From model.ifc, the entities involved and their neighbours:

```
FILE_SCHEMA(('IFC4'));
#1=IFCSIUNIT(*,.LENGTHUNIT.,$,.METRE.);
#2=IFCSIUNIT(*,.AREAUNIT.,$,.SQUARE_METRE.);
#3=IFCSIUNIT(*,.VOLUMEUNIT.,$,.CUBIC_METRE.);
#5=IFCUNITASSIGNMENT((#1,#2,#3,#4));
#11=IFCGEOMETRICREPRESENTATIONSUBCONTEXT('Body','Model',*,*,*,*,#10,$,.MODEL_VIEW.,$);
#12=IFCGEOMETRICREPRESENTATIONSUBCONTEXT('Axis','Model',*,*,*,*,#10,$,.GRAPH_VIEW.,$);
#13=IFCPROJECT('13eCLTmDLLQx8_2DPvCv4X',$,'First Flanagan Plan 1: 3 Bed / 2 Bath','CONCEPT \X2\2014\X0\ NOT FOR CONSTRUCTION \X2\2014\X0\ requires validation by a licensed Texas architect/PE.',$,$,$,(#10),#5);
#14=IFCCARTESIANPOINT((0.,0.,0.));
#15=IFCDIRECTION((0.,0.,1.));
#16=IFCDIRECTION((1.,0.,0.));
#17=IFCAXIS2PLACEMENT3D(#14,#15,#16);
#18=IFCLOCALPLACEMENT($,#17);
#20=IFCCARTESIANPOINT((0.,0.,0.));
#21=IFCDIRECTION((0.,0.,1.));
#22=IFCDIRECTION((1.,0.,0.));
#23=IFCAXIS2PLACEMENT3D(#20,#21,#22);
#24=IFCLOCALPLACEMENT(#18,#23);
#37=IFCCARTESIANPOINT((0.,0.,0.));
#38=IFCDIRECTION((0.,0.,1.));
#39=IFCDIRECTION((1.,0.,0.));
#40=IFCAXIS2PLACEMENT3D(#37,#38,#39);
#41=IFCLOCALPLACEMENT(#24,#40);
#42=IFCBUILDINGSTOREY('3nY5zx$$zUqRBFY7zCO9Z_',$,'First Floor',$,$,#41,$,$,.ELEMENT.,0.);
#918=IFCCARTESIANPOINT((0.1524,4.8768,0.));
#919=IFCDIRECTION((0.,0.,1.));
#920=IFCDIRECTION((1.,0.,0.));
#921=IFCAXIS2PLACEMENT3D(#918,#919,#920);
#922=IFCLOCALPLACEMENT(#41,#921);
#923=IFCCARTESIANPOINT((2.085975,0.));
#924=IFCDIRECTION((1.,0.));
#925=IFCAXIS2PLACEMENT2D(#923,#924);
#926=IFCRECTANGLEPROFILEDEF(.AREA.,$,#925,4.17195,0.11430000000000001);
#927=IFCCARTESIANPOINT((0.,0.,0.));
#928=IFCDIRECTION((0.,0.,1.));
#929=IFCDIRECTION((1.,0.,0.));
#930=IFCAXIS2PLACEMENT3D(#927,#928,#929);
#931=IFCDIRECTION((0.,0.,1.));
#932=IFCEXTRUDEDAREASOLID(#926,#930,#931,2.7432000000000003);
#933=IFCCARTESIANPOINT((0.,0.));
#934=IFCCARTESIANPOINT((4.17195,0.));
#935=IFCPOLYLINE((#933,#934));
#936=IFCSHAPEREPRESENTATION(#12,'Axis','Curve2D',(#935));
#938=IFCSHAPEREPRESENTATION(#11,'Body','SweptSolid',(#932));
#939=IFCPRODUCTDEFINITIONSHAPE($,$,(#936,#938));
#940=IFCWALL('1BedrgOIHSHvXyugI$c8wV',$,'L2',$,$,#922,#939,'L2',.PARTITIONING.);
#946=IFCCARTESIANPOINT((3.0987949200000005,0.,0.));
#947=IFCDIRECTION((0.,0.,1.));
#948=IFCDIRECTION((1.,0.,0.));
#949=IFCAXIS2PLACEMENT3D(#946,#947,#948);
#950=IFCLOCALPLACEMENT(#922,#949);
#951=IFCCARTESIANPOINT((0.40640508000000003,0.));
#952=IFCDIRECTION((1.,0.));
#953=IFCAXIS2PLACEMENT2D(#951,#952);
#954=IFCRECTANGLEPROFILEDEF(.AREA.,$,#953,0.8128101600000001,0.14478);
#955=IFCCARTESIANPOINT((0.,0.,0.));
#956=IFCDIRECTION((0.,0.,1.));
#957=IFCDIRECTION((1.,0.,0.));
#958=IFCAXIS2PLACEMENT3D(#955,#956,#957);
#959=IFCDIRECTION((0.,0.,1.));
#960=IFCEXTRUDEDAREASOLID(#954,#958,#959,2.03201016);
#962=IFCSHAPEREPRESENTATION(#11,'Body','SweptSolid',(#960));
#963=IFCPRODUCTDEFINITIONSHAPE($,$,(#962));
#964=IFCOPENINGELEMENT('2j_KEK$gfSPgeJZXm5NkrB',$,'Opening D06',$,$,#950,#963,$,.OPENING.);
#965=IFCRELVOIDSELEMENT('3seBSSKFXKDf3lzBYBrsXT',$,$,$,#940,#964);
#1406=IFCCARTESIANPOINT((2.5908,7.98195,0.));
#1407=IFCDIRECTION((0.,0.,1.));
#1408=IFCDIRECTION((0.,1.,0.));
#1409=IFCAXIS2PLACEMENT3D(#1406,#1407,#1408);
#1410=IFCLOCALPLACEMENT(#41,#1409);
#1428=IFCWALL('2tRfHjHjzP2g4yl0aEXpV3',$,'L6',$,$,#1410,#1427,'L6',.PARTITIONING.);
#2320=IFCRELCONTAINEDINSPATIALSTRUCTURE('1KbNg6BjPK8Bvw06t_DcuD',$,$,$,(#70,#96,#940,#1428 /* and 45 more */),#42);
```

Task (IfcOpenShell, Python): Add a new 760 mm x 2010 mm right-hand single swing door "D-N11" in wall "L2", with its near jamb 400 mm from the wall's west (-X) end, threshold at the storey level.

```python
import numpy as np
import ifcopenshell
import ifcopenshell.api.feature
import ifcopenshell.api.geometry
import ifcopenshell.api.root
import ifcopenshell.api.spatial
import ifcopenshell.geom
import ifcopenshell.util.element
import ifcopenshell.util.placement
import ifcopenshell.util.representation
import ifcopenshell.util.shape
import ifcopenshell.util.unit

model = ifcopenshell.open("model.ifc")
unit_scale = ifcopenshell.util.unit.calculate_unit_scale(model)
settings = ifcopenshell.geom.settings()


def volume(element):
    """Net volume in cubic metres, openings subtracted."""
    shape = ifcopenshell.geom.create_shape(settings, element)
    return ifcopenshell.util.shape.get_volume(shape.geometry)


wall = model.by_guid("1BedrgOIHSHvXyugI$c8wV")
storey = ifcopenshell.util.element.get_container(wall, ifc_class="IfcBuildingStorey")
context = ifcopenshell.util.representation.get_context(model, "Model", "Body", "MODEL_VIEW")
before = volume(wall)

width, height, from_end, sill = 0.76, 2.01, 0.4, 0.0  # metres

# The wall runs along its own X axis, and the end named is its -X end.
wall_shape = ifcopenshell.geom.create_shape(settings, wall)
x, y, z = ifcopenshell.util.shape.get_vertices(wall_shape.geometry).T
start = x.min() + from_end
face, thickness = float(y.min()), float(y.max() - y.min())
wall_matrix = ifcopenshell.util.placement.get_local_placement(wall.ObjectPlacement)
level = ifcopenshell.util.placement.get_local_placement(storey.ObjectPlacement)[2, 3]


def in_wall(x, y):
    """Placement at x, y metres in the wall's axes, at sill height."""
    matrix = wall_matrix.copy()
    matrix[:, 3] = wall_matrix @ np.array([x / unit_scale, y / unit_scale, 0.0, 1.0])
    matrix[2, 3] = level + sill / unit_scale
    return matrix


# Opening: a box that overshoots both wall faces by 50 mm.
opening = ifcopenshell.api.root.create_entity(model, ifc_class="IfcOpeningElement", predefined_type="OPENING")
box = ifcopenshell.api.geometry.add_wall_representation(
    model, context=context, length=width, height=height, thickness=thickness + 0.1
)
ifcopenshell.api.geometry.assign_representation(model, product=opening, representation=box)
ifcopenshell.api.geometry.edit_object_placement(model, product=opening, matrix=in_wall(start, face - 0.05), is_si=False)
ifcopenshell.api.feature.add_feature(model, feature=opening, element=wall)

door = ifcopenshell.api.root.create_entity(model, ifc_class="IfcDoor", name="D-N11", predefined_type="DOOR")
door.OverallWidth, door.OverallHeight = width / unit_scale, height / unit_scale
door.OperationType = "SINGLE_SWING_RIGHT"
body = ifcopenshell.api.geometry.add_door_representation(
    model,
    context=context,
    overall_width=door.OverallWidth,
    overall_height=door.OverallHeight,
    operation_type="SINGLE_SWING_RIGHT",
    lining_properties={"LiningDepth": thickness / unit_scale, "ThresholdDepth": thickness / unit_scale},
)
ifcopenshell.api.geometry.assign_representation(model, product=door, representation=body)
ifcopenshell.api.spatial.assign_container(model, products=[door], relating_structure=storey)
ifcopenshell.api.feature.add_filling(model, opening=opening, element=door)

# The lining spans the wall, so the door starts at the wall face.
ifcopenshell.api.geometry.edit_object_placement(model, product=door, matrix=in_wall(start, face), is_si=False)

after = volume(wall)

print(f"wall volume {before:.3f} -> {after:.3f} m3")

model.write("model-out.ifc")
```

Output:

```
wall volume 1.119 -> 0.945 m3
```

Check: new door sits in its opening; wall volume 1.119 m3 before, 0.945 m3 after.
